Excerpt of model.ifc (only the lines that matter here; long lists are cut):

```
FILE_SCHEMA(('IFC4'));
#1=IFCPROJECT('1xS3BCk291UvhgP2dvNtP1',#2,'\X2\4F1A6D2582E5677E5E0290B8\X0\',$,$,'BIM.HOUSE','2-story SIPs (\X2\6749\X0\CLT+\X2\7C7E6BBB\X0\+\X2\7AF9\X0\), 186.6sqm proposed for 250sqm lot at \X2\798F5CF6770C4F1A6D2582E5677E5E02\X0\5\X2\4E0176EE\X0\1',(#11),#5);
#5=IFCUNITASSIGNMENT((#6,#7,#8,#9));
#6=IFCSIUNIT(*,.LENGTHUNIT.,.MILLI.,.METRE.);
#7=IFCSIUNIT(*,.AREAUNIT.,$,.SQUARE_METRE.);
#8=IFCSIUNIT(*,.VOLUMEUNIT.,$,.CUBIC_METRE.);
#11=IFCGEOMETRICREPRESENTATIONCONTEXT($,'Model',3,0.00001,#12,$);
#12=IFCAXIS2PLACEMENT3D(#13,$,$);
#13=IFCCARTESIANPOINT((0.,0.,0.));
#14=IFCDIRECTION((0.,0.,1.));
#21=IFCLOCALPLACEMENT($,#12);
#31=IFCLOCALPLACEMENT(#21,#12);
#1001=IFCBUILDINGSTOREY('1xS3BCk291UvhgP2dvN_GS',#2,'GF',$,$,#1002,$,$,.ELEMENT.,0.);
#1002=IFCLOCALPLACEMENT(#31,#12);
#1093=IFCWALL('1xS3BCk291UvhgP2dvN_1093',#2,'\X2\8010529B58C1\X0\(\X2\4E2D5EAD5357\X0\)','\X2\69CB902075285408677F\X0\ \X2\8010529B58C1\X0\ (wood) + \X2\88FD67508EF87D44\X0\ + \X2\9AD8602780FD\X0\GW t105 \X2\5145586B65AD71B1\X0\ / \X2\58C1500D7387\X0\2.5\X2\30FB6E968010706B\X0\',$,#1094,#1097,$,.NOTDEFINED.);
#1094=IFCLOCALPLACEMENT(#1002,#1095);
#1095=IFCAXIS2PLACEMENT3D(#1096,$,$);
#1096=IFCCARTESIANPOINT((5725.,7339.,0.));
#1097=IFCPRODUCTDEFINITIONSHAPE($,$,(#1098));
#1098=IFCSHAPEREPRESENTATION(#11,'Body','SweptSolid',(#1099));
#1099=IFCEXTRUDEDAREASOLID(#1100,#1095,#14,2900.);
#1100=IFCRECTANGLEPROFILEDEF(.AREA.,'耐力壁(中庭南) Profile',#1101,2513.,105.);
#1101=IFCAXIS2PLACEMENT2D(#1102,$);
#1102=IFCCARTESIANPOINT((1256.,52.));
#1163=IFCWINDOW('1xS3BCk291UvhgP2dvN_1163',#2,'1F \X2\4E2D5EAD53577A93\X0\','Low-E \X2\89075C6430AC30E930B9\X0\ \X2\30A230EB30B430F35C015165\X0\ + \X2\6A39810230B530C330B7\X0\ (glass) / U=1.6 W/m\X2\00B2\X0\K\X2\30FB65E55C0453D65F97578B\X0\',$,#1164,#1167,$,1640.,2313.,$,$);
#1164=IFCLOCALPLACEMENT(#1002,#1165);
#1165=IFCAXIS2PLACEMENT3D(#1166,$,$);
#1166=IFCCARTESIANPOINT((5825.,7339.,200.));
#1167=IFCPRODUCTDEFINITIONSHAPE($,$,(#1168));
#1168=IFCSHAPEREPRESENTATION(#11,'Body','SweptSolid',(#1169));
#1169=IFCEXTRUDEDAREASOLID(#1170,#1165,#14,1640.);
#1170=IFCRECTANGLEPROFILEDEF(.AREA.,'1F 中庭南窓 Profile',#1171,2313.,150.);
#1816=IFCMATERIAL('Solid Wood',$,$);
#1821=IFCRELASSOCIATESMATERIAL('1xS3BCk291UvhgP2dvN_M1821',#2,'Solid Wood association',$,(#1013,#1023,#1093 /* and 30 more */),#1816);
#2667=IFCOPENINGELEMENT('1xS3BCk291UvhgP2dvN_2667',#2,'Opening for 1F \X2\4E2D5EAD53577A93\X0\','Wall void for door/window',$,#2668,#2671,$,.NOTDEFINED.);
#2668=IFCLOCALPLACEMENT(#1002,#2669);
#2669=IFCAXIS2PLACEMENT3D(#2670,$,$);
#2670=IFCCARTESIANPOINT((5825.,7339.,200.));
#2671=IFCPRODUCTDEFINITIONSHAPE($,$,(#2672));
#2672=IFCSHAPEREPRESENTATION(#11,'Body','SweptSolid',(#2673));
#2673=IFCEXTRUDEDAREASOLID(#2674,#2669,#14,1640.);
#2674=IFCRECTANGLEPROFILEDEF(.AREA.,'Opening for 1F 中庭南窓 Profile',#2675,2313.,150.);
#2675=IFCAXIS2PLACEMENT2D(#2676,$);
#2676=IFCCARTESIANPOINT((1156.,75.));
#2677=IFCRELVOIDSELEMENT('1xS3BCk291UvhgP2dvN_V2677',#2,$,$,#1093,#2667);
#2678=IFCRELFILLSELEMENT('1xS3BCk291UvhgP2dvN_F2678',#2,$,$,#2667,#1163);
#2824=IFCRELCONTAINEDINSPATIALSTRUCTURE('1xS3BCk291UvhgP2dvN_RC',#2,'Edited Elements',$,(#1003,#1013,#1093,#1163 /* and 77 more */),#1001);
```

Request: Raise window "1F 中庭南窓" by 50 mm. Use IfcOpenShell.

```python
import numpy as np
import ifcopenshell
import ifcopenshell.api.geometry
import ifcopenshell.util.placement
import ifcopenshell.util.unit

model = ifcopenshell.open("model.ifc")
unit_scale = ifcopenshell.util.unit.calculate_unit_scale(model)

window = model.by_guid("1xS3BCk291UvhgP2dvN_1163")
opening = window.FillsVoids[0].RelatingOpeningElement
dz = 0.05 / unit_scale

shift = np.array([0.0, 0.0, dz])
# The window is not placed relative to its opening, so move both.
for product in (opening, window):
    matrix = ifcopenshell.util.placement.get_local_placement(product.ObjectPlacement)
    matrix[:3, 3] += shift
    ifcopenshell.api.geometry.edit_object_placement(model, product=product, matrix=matrix, is_si=False)

print(f"moved by {dz * unit_scale:+.3f} m")

model.write("model-out.ifc")
```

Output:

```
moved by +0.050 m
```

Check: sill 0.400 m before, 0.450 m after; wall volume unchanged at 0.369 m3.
